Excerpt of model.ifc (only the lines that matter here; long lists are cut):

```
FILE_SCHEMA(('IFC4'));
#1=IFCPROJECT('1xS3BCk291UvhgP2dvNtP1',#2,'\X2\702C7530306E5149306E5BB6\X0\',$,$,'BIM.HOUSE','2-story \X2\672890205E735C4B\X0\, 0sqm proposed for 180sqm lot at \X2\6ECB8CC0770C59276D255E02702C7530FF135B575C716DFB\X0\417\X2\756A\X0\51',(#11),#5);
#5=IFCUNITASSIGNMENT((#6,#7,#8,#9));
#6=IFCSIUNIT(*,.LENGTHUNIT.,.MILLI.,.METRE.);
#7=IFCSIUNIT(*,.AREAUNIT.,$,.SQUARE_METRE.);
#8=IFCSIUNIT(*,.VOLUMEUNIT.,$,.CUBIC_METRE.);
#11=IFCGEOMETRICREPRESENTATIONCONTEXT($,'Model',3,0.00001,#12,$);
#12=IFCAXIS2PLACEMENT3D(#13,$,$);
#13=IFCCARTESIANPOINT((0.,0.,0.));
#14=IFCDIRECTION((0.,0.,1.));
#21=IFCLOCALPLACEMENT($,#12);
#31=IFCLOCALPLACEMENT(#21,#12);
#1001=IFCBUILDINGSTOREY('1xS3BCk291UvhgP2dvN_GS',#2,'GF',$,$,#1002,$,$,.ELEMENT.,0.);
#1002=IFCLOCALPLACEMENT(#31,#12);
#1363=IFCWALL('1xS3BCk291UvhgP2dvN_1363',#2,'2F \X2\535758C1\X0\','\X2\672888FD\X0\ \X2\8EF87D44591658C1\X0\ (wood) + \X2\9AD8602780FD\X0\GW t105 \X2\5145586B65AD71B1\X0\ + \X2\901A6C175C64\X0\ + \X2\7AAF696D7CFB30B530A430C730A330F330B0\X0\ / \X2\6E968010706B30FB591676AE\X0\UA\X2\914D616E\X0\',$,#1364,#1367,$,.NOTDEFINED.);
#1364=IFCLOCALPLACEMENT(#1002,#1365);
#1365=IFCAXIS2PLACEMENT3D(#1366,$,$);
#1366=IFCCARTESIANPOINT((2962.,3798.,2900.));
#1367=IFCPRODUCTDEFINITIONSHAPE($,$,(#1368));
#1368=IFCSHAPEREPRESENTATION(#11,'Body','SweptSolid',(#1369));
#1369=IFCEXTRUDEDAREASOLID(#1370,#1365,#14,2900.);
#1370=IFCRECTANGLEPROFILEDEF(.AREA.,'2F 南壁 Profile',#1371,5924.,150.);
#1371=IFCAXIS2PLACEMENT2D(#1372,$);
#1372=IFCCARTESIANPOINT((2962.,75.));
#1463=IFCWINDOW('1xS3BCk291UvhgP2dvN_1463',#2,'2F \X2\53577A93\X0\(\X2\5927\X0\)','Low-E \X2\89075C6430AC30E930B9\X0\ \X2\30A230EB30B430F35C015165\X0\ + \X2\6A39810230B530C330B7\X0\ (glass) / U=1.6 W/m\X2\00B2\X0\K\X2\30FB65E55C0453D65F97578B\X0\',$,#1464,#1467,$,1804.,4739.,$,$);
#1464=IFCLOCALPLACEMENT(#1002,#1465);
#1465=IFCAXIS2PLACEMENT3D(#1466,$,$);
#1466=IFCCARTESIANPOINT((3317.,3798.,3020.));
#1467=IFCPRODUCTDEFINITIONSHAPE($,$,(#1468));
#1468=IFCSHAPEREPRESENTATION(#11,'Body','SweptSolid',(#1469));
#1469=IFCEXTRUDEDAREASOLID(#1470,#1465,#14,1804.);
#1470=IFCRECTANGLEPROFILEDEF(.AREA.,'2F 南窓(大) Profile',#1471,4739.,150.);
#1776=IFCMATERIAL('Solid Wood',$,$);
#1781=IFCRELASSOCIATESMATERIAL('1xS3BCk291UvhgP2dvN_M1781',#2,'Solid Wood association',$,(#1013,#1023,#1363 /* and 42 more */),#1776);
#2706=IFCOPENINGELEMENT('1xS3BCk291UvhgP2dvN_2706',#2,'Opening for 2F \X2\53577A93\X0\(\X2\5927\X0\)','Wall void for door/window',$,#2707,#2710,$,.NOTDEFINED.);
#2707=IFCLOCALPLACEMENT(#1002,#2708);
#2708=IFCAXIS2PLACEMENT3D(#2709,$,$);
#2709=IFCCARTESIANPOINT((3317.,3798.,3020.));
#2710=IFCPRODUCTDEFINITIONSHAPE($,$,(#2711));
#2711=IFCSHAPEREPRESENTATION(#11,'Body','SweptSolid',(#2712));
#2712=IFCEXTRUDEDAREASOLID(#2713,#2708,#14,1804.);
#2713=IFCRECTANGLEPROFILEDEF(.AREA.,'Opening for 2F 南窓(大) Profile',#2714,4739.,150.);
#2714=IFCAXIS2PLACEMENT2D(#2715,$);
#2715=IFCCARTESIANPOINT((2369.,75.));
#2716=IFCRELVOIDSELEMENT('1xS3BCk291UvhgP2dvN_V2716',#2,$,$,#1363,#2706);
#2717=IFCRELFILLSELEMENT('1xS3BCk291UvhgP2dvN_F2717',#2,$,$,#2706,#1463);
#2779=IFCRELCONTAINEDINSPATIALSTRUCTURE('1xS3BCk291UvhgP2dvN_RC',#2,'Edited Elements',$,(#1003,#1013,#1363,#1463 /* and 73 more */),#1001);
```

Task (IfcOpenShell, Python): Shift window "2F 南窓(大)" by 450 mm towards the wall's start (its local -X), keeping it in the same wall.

```python
import ifcopenshell
import ifcopenshell.api.geometry
import ifcopenshell.util.placement
import ifcopenshell.util.unit

model = ifcopenshell.open("model.ifc")
unit_scale = ifcopenshell.util.unit.calculate_unit_scale(model)

window = model.by_guid("1xS3BCk291UvhgP2dvN_1463")
opening = window.FillsVoids[0].RelatingOpeningElement
wall = opening.VoidsElements[0].RelatingBuildingElement

wall_matrix = ifcopenshell.util.placement.get_local_placement(wall.ObjectPlacement)
shift = wall_matrix[:3, 0] * -0.45 / unit_scale
before = ifcopenshell.util.placement.get_local_placement(window.ObjectPlacement)[:3, 3].copy()

# The window is not placed relative to its opening, so move both.
for product in (opening, window):
    matrix = ifcopenshell.util.placement.get_local_placement(product.ObjectPlacement)
    matrix[:3, 3] += shift
    ifcopenshell.api.geometry.edit_object_placement(model, product=product, matrix=matrix, is_si=False)

after = ifcopenshell.util.placement.get_local_placement(window.ObjectPlacement)[:3, 3]
print("window moved by", (after - before).round(3) + 0.0)

model.write("model_v2.ifc")
```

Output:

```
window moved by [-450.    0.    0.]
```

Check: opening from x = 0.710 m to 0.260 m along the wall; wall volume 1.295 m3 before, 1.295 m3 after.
